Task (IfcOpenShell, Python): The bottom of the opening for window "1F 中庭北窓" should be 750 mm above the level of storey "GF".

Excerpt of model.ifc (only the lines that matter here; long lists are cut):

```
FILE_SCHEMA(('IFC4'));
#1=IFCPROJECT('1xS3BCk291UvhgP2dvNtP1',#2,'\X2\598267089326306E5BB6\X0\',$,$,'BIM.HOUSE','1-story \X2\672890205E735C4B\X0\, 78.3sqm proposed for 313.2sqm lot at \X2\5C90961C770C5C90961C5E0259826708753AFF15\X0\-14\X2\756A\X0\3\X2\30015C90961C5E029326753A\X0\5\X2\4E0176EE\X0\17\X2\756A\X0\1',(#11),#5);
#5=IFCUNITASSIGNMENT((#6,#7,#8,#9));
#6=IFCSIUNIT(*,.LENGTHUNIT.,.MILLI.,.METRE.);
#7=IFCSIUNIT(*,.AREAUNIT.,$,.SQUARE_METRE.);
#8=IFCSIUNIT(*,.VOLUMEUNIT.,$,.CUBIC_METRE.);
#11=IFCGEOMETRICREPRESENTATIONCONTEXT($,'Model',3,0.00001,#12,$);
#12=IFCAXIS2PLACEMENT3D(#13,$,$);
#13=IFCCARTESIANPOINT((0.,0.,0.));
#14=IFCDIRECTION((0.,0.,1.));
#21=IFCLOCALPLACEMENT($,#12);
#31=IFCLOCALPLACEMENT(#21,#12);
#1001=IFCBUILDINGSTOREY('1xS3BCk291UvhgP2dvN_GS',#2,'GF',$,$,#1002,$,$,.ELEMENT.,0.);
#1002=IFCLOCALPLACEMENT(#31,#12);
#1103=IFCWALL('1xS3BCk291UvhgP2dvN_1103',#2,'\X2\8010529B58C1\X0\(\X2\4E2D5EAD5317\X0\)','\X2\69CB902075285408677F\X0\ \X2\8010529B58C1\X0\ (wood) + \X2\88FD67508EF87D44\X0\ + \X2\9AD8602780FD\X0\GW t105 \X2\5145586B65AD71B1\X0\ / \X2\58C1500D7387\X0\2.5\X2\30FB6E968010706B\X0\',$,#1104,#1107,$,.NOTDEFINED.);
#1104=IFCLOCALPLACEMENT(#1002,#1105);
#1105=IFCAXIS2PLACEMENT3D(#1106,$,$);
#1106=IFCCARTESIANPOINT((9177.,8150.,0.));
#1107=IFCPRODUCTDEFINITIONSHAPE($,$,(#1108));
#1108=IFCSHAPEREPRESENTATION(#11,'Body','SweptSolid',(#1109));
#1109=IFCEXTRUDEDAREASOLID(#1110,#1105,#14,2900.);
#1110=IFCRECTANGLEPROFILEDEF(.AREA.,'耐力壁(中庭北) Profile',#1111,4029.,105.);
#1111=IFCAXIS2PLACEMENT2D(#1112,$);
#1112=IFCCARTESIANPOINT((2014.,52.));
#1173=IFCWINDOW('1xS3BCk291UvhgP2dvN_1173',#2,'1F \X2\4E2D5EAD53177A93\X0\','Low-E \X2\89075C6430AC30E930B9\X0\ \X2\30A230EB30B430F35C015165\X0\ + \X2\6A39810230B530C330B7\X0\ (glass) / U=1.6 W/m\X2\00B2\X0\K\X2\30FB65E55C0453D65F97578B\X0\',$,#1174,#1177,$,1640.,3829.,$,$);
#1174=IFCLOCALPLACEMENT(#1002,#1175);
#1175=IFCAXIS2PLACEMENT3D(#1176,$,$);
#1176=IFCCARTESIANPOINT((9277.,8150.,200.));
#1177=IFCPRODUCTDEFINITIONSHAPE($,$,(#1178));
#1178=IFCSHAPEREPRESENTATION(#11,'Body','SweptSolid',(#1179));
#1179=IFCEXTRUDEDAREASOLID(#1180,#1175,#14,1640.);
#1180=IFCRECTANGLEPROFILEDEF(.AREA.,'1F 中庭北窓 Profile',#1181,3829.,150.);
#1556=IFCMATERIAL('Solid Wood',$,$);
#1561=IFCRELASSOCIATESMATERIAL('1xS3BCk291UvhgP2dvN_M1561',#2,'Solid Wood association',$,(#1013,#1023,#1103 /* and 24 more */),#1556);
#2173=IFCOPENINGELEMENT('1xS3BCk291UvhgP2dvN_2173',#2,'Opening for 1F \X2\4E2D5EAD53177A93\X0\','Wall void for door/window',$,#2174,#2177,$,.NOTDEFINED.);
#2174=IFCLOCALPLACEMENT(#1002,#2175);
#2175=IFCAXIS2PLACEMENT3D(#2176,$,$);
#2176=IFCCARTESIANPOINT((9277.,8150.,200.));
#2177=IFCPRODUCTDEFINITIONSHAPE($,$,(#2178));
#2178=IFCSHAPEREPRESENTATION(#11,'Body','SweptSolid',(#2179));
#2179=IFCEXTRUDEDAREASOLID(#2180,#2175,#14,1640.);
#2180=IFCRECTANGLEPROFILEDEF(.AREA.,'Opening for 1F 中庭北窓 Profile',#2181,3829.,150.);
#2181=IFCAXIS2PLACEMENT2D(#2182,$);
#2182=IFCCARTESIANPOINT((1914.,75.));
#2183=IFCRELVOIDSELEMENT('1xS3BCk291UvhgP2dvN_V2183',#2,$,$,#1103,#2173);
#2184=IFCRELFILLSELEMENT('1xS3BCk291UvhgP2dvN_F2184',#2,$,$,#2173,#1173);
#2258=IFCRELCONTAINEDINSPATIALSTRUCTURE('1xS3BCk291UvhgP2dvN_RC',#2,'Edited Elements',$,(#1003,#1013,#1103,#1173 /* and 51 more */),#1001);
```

```python
import numpy as np
import ifcopenshell
import ifcopenshell.api.geometry
import ifcopenshell.geom
import ifcopenshell.util.element
import ifcopenshell.util.placement
import ifcopenshell.util.shape
import ifcopenshell.util.unit

model = ifcopenshell.open("model.ifc")
unit_scale = ifcopenshell.util.unit.calculate_unit_scale(model)

window = model.by_guid("1xS3BCk291UvhgP2dvN_1173")
opening = window.FillsVoids[0].RelatingOpeningElement
storey = ifcopenshell.util.element.get_container(window, ifc_class="IfcBuildingStorey")
level = ifcopenshell.util.placement.get_local_placement(storey.ObjectPlacement)[2, 3]

# The opening's origin need not be at the sill, so measure its lowest point.
shape = ifcopenshell.geom.create_shape(ifcopenshell.geom.settings(), opening)
bottom = ifcopenshell.util.shape.get_shape_bottom_elevation(shape, shape.geometry) / unit_scale
dz = level + 0.75 / unit_scale - bottom

shift = np.array([0.0, 0.0, dz])
# The window is not placed relative to its opening, so move both.
for product in (opening, window):
    matrix = ifcopenshell.util.placement.get_local_placement(product.ObjectPlacement)
    matrix[:3, 3] += shift
    ifcopenshell.api.geometry.edit_object_placement(model, product=product, matrix=matrix, is_si=False)

print(f"moved by {dz * unit_scale:+.3f} m")

model.write("model_v2.ifc")
```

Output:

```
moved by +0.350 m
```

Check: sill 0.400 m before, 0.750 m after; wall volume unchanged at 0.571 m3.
